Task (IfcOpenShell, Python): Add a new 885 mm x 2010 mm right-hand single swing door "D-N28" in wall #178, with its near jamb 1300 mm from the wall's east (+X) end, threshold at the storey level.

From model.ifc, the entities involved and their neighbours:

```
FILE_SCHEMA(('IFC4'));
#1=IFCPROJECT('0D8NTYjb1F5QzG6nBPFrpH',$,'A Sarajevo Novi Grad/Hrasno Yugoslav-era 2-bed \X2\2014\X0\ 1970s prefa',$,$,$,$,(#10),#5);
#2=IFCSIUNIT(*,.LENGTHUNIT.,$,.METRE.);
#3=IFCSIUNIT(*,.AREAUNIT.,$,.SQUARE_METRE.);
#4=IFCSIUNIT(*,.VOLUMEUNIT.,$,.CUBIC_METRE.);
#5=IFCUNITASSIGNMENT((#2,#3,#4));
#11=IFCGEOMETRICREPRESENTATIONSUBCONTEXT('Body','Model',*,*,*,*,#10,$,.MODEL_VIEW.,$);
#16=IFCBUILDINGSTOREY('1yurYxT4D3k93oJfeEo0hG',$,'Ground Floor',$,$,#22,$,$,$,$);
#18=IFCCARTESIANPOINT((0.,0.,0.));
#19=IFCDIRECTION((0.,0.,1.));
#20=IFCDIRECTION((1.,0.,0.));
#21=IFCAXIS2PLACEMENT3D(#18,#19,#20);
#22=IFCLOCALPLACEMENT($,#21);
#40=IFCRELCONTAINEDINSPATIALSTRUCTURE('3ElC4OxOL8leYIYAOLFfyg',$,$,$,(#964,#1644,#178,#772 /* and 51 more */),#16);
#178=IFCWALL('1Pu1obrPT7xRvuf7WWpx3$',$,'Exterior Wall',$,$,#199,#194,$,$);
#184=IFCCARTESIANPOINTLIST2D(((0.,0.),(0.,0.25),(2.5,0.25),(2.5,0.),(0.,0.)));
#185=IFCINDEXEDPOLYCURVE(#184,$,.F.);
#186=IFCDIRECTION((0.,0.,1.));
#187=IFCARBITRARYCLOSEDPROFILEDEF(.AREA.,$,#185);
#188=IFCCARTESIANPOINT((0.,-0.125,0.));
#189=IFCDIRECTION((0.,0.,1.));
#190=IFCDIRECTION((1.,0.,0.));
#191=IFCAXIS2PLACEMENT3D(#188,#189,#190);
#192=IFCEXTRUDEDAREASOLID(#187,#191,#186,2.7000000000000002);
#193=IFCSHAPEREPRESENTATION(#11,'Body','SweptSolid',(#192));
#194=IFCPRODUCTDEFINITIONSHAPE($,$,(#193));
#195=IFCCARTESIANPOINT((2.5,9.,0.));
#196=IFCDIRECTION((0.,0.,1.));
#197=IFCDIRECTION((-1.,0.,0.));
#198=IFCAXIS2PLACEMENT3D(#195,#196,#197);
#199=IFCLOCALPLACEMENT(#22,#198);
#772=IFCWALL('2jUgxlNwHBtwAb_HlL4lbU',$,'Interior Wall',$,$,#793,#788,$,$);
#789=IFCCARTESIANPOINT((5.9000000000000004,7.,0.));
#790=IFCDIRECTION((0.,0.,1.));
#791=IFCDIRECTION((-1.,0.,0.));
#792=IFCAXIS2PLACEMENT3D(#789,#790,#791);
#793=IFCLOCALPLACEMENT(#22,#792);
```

```python
import numpy as np
import ifcopenshell
import ifcopenshell.api.feature
import ifcopenshell.api.geometry
import ifcopenshell.api.root
import ifcopenshell.api.spatial
import ifcopenshell.geom
import ifcopenshell.util.element
import ifcopenshell.util.placement
import ifcopenshell.util.representation
import ifcopenshell.util.shape
import ifcopenshell.util.unit

model = ifcopenshell.open("model.ifc")
unit_scale = ifcopenshell.util.unit.calculate_unit_scale(model)
settings = ifcopenshell.geom.settings()


def volume(element):
    """Net volume in cubic metres, openings subtracted."""
    shape = ifcopenshell.geom.create_shape(settings, element)
    return ifcopenshell.util.shape.get_volume(shape.geometry)


wall = model.by_guid("1Pu1obrPT7xRvuf7WWpx3$")
storey = ifcopenshell.util.element.get_container(wall, ifc_class="IfcBuildingStorey")
context = ifcopenshell.util.representation.get_context(model, "Model", "Body", "MODEL_VIEW")
before = volume(wall)

width, height, from_end, sill = 0.885, 2.01, 1.3, 0.0  # metres

# The wall runs along its own X axis, and the end named is its -X end.
wall_shape = ifcopenshell.geom.create_shape(settings, wall)
x, y, z = ifcopenshell.util.shape.get_vertices(wall_shape.geometry).T
start = x.min() + from_end
face, thickness = float(y.min()), float(y.max() - y.min())
wall_matrix = ifcopenshell.util.placement.get_local_placement(wall.ObjectPlacement)
level = ifcopenshell.util.placement.get_local_placement(storey.ObjectPlacement)[2, 3]


def in_wall(x, y):
    """Placement at x, y metres in the wall's axes, at sill height."""
    matrix = wall_matrix.copy()
    matrix[:, 3] = wall_matrix @ np.array([x / unit_scale, y / unit_scale, 0.0, 1.0])
    matrix[2, 3] = level + sill / unit_scale
    return matrix


# Opening: a box that overshoots both wall faces by 50 mm.
opening = ifcopenshell.api.root.create_entity(model, ifc_class="IfcOpeningElement", predefined_type="OPENING")
box = ifcopenshell.api.geometry.add_wall_representation(
    model, context=context, length=width, height=height, thickness=thickness + 0.1
)
ifcopenshell.api.geometry.assign_representation(model, product=opening, representation=box)
ifcopenshell.api.geometry.edit_object_placement(model, product=opening, matrix=in_wall(start, face - 0.05), is_si=False)
ifcopenshell.api.feature.add_feature(model, feature=opening, element=wall)

door = ifcopenshell.api.root.create_entity(model, ifc_class="IfcDoor", name="D-N28", predefined_type="DOOR")
door.OverallWidth, door.OverallHeight = width / unit_scale, height / unit_scale
door.OperationType = "SINGLE_SWING_RIGHT"
body = ifcopenshell.api.geometry.add_door_representation(
    model,
    context=context,
    overall_width=door.OverallWidth,
    overall_height=door.OverallHeight,
    operation_type="SINGLE_SWING_RIGHT",
    lining_properties={"LiningDepth": thickness / unit_scale, "ThresholdDepth": thickness / unit_scale},
)
ifcopenshell.api.geometry.assign_representation(model, product=door, representation=body)
ifcopenshell.api.spatial.assign_container(model, products=[door], relating_structure=storey)
ifcopenshell.api.feature.add_filling(model, opening=opening, element=door)

# The lining spans the wall, so the door starts at the wall face.
ifcopenshell.api.geometry.edit_object_placement(model, product=door, matrix=in_wall(start, face), is_si=False)

after = volume(wall)

print(f"wall volume {before:.3f} -> {after:.3f} m3")

model.write("model_v2.ifc")
```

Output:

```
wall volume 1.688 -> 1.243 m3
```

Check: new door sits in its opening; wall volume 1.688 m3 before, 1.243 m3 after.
